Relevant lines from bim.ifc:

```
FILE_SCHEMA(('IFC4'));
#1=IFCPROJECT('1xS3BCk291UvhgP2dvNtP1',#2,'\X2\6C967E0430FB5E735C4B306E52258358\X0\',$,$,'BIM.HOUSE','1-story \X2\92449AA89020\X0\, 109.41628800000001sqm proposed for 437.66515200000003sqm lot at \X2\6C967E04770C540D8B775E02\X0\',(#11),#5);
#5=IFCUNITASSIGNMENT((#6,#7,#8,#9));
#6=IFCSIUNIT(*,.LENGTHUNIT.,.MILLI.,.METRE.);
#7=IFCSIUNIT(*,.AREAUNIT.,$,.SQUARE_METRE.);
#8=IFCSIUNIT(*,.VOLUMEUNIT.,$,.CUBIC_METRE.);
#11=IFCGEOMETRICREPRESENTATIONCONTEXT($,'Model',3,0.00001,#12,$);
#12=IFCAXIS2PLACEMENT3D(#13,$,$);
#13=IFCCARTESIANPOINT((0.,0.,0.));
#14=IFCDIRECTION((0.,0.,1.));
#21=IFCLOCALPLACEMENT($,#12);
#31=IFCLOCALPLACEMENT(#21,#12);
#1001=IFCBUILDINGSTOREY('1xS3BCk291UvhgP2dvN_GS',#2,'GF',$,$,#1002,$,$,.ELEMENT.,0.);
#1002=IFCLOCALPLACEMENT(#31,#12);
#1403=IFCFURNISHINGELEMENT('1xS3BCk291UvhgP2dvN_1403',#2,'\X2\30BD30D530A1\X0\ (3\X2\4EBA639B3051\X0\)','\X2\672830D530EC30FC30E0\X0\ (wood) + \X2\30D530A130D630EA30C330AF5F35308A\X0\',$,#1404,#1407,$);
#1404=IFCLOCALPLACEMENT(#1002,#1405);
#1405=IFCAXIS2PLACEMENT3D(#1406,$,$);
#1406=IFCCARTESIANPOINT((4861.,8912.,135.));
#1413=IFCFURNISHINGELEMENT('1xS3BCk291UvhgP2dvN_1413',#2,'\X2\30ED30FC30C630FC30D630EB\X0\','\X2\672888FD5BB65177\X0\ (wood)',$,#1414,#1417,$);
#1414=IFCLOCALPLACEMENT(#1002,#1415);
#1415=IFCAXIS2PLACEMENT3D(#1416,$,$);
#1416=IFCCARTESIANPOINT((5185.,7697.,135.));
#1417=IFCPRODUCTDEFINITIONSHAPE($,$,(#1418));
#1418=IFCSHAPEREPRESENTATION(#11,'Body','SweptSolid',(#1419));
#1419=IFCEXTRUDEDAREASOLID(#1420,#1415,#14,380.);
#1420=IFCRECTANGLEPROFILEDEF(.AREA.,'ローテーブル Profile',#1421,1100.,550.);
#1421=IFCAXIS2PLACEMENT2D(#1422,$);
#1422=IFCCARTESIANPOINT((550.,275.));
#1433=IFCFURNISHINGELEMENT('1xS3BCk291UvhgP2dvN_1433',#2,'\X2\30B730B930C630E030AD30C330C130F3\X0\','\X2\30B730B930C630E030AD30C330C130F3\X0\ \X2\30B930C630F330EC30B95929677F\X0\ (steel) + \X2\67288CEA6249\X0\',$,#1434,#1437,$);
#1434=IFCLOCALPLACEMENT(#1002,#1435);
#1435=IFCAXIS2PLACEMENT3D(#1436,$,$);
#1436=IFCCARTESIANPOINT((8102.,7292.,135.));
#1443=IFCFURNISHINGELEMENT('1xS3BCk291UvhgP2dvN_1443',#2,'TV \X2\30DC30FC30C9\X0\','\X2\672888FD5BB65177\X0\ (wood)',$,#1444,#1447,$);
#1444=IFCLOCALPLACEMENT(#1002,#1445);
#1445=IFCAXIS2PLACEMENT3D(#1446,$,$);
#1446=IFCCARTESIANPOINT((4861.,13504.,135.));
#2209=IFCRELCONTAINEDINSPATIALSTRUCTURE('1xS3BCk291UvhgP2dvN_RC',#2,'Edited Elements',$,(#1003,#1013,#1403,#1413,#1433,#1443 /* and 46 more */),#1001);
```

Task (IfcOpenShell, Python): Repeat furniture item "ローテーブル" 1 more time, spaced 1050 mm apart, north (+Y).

```python
import numpy as np
import ifcopenshell
import ifcopenshell.api.geometry
import ifcopenshell.api.root
import ifcopenshell.util.element
import ifcopenshell.util.placement

model = ifcopenshell.open("bim.ifc")


def reuse_history(source, copy):
    """copy_class also copies each property set's owner history, people and application; keep the originals."""
    for rel in copy.IsDefinedBy:
        if rel.is_a("IfcRelDefinesByProperties") and (history := rel.RelatingPropertyDefinition.OwnerHistory):
            rel.RelatingPropertyDefinition.OwnerHistory = source.OwnerHistory
            ifcopenshell.util.element.remove_deep2(model, history)


source = model.by_guid("1xS3BCk291UvhgP2dvN_1413")
base = ifcopenshell.util.placement.get_local_placement(source.ObjectPlacement)
step = np.array([0.0, 1.0, 0.0]) * 1050.0

for i in range(1, 2):
    copy = ifcopenshell.api.root.copy_class(model, product=source)
    copy.Representation = ifcopenshell.util.element.copy_deep(
        model, source.Representation, exclude=["IfcGeometricRepresentationContext", "IfcRepresentationMap"]
    )
    reuse_history(source, copy)
    matrix = base.copy()
    matrix[:3, 3] += i * step
    print("added at", matrix[:3, 3].round(3) + 0.0)
    ifcopenshell.api.geometry.edit_object_placement(model, product=copy, matrix=matrix, is_si=False)

model.write("bim-out.ifc")
```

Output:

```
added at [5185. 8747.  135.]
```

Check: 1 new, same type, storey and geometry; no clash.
